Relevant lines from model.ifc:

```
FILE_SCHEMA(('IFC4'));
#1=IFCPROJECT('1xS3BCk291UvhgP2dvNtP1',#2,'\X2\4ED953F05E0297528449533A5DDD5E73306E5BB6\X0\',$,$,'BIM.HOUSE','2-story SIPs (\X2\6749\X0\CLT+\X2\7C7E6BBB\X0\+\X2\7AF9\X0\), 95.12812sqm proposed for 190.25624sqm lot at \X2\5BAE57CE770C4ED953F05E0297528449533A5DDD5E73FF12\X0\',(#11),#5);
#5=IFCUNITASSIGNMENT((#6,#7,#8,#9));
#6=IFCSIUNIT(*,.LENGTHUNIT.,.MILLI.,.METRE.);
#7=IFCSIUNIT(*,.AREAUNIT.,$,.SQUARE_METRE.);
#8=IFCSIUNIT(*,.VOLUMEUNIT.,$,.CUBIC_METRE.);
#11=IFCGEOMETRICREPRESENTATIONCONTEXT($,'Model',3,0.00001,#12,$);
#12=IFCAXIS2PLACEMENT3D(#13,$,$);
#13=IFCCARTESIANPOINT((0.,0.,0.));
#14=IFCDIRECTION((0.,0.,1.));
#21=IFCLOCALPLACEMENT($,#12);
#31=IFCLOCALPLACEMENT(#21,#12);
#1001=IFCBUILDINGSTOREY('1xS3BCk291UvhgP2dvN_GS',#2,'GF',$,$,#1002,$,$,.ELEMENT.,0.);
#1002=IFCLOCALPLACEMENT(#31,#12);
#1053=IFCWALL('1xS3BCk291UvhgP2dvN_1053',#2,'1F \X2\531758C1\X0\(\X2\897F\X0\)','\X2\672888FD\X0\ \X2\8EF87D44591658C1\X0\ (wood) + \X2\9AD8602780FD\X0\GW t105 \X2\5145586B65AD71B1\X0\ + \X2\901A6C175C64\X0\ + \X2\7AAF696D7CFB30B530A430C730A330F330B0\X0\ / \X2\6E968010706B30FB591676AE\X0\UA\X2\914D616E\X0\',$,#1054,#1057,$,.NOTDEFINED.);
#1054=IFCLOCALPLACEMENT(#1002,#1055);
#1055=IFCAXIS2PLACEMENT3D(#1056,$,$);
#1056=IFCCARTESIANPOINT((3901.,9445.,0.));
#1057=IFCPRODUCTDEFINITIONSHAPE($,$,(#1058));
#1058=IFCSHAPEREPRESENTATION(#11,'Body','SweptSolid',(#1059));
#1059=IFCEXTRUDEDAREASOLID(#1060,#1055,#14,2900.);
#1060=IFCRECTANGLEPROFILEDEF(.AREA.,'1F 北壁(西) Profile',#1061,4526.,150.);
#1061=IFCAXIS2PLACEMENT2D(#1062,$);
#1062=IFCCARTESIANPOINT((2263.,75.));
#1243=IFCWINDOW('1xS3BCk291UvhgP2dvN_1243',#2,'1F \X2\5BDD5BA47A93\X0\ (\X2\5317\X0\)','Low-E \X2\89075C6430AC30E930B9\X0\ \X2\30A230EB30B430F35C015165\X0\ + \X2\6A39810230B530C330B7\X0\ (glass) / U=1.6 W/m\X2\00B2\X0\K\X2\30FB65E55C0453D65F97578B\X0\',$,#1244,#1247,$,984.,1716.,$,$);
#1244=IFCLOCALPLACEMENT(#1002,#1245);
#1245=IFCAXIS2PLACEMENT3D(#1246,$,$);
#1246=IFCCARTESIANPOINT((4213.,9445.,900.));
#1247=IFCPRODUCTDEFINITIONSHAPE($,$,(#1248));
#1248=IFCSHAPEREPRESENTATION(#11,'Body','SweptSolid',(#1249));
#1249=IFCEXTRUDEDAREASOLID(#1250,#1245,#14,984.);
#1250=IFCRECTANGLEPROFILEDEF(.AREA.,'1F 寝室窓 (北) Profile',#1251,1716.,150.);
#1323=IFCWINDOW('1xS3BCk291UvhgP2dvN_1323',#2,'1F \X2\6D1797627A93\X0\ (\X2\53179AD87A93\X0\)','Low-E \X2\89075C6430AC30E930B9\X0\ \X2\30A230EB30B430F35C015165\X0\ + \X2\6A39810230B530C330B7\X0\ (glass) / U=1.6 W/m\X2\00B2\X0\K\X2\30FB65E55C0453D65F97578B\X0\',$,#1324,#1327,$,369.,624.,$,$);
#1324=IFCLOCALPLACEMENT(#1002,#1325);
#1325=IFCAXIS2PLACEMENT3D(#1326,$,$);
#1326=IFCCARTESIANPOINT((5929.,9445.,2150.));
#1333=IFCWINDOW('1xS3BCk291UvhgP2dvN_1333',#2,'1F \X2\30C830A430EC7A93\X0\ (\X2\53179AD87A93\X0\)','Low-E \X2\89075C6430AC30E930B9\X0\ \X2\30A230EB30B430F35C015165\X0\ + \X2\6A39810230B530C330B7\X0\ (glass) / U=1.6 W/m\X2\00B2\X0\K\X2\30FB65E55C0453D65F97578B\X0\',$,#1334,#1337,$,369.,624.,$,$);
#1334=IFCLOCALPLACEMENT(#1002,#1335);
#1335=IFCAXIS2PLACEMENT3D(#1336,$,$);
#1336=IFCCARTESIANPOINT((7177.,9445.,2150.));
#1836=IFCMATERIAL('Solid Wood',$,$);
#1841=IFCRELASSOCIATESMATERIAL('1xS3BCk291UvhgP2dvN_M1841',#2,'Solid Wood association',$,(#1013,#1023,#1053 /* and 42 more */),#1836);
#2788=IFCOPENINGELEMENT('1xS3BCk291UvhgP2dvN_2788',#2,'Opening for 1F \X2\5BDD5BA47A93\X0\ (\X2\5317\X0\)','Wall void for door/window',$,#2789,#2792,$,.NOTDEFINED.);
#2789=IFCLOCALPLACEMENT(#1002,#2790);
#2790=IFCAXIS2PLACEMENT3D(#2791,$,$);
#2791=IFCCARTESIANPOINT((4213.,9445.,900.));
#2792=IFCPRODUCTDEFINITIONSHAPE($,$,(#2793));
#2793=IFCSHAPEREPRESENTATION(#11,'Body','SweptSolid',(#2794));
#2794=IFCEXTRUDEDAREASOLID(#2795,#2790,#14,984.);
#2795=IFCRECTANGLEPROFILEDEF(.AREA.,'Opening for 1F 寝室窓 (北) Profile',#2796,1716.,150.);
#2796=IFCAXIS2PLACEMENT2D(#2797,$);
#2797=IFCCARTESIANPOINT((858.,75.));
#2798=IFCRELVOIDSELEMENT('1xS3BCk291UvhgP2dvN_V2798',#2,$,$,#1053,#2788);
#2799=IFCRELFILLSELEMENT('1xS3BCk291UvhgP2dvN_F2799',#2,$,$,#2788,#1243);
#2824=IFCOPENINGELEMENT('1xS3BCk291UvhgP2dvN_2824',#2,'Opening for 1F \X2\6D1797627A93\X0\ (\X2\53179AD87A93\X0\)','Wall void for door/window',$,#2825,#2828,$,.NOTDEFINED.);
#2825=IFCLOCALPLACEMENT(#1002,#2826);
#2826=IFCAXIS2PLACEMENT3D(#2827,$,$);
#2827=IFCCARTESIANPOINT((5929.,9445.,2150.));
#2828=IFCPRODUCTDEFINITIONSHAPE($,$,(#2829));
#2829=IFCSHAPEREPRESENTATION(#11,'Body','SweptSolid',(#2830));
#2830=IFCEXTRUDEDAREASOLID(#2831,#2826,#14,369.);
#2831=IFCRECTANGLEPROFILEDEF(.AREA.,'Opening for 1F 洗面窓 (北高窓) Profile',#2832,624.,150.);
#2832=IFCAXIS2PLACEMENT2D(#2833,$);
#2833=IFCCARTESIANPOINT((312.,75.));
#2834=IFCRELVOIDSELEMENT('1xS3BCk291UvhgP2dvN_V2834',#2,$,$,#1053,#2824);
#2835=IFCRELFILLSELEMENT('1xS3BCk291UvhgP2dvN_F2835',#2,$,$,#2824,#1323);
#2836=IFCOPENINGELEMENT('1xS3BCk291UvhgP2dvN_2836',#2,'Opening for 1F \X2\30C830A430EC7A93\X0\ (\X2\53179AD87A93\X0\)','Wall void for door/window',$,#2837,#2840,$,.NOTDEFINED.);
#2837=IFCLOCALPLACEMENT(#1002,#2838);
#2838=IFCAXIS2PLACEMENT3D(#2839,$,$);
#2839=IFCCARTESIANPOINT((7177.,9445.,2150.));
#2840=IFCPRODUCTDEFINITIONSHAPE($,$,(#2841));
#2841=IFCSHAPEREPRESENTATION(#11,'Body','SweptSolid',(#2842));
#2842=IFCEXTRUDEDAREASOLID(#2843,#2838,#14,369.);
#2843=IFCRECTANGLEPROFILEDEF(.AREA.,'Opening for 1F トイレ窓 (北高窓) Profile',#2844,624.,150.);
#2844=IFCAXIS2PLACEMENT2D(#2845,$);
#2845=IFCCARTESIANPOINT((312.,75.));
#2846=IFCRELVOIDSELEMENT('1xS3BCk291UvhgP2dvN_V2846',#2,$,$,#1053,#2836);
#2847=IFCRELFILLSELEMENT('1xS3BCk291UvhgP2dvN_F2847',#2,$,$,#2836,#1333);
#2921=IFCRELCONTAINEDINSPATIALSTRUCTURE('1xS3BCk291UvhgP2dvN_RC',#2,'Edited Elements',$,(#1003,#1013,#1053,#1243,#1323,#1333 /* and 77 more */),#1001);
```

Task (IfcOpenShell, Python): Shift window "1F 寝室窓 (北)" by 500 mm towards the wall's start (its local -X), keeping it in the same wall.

```python
import ifcopenshell
import ifcopenshell.api.geometry
import ifcopenshell.util.placement
import ifcopenshell.util.unit

model = ifcopenshell.open("model.ifc")
unit_scale = ifcopenshell.util.unit.calculate_unit_scale(model)

window = model.by_guid("1xS3BCk291UvhgP2dvN_1243")
opening = window.FillsVoids[0].RelatingOpeningElement
wall = opening.VoidsElements[0].RelatingBuildingElement

wall_matrix = ifcopenshell.util.placement.get_local_placement(wall.ObjectPlacement)
shift = wall_matrix[:3, 0] * -0.5 / unit_scale
before = ifcopenshell.util.placement.get_local_placement(window.ObjectPlacement)[:3, 3].copy()

# The window is not placed relative to its opening, so move both.
for product in (opening, window):
    matrix = ifcopenshell.util.placement.get_local_placement(product.ObjectPlacement)
    matrix[:3, 3] += shift
    ifcopenshell.api.geometry.edit_object_placement(model, product=product, matrix=matrix, is_si=False)

after = ifcopenshell.util.placement.get_local_placement(window.ObjectPlacement)[:3, 3]
print("window moved by", (after - before).round(3) + 0.0)

model.write("model_edited.ifc")
```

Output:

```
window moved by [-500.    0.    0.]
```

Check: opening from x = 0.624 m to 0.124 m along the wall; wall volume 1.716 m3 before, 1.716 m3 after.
